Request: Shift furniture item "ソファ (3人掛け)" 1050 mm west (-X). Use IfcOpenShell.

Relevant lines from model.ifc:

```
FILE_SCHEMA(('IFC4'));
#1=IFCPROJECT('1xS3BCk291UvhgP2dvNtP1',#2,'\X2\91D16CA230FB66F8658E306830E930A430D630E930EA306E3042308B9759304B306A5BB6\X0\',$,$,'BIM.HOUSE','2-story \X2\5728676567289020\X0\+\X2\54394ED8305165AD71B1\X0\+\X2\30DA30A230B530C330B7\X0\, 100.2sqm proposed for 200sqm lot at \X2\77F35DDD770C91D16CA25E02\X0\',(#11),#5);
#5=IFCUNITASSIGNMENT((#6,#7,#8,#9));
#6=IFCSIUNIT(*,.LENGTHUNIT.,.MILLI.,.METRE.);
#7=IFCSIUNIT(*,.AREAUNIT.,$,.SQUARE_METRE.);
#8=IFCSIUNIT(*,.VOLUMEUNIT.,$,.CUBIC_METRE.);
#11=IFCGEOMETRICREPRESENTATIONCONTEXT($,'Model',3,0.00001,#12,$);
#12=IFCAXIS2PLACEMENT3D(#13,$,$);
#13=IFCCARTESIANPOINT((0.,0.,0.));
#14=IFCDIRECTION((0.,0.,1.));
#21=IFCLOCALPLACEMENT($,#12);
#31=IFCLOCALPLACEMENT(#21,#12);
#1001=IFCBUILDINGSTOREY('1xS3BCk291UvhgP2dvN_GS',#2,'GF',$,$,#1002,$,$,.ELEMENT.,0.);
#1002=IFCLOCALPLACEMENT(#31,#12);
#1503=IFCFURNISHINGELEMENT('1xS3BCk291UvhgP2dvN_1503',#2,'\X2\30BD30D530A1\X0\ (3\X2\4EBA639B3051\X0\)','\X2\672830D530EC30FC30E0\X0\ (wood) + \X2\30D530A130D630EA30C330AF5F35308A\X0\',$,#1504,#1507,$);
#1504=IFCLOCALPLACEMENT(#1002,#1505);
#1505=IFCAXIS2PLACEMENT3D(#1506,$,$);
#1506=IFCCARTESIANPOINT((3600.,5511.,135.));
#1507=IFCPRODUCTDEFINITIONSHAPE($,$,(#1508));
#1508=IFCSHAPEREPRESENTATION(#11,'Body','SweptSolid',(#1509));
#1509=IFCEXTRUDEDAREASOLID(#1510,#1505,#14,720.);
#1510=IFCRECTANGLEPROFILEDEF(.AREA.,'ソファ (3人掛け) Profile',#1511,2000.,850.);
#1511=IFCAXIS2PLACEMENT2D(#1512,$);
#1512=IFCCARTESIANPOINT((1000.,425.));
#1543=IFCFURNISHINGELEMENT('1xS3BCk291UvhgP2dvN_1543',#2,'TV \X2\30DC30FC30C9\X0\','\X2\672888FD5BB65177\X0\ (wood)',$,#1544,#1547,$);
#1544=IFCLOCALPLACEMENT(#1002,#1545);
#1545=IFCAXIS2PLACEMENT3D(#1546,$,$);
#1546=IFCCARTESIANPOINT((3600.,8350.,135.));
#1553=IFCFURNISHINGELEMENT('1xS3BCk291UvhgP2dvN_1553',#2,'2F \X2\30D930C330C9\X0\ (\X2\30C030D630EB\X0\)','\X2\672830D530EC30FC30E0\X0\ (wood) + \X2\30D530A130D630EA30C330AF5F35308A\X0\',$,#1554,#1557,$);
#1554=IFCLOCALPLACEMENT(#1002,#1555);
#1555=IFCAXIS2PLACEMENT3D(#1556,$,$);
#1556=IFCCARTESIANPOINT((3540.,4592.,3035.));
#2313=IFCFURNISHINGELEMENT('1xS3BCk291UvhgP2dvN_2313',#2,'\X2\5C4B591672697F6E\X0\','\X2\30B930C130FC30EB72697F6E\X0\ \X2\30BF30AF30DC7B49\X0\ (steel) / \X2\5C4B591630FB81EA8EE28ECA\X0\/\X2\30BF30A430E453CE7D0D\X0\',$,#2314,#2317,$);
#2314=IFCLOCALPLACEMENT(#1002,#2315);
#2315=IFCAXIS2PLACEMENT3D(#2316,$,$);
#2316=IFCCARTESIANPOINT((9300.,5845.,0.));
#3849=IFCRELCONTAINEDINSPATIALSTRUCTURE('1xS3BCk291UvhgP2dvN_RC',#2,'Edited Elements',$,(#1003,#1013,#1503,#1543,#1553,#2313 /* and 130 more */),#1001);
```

```python
import ifcopenshell
import ifcopenshell.api.geometry
import ifcopenshell.util.placement
import ifcopenshell.util.unit

model = ifcopenshell.open("model.ifc")
unit_scale = ifcopenshell.util.unit.calculate_unit_scale(model)

item = model.by_guid("1xS3BCk291UvhgP2dvN_1503")
matrix = ifcopenshell.util.placement.get_local_placement(item.ObjectPlacement)
matrix[0, 3] -= 1.05 / unit_scale
ifcopenshell.api.geometry.edit_object_placement(model, product=item, matrix=matrix, is_si=False)

print(ifcopenshell.util.placement.get_local_placement(item.ObjectPlacement).round(3) + 0.0)

model.write("model_updated.ifc")
```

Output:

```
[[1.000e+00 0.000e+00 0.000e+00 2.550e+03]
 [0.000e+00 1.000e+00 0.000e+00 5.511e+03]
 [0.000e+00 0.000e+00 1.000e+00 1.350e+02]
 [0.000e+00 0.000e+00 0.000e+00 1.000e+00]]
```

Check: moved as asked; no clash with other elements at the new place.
